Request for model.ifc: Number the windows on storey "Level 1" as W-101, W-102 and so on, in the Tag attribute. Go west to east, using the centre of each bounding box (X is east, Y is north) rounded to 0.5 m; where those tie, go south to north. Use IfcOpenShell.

First a look at what the model holds.

```python
import ifcopenshell
import ifcopenshell.util.element
import ifcopenshell.util.placement

model = ifcopenshell.open("model.ifc")
print(model.schema)
storey = next(s for s in model.by_type("IfcBuildingStorey") if s.Name == "Level 1")
windows = [e for e in ifcopenshell.util.element.get_decomposition(storey) if e.is_a("IfcWindow")]
for e in sorted(windows, key=lambda e: e.id()):
    origin = ifcopenshell.util.placement.get_local_placement(e.ObjectPlacement)[:3, 3]
    print(e.id(), e.Tag, e.Name, origin.round(2) + 0.0, sep=" | ")
```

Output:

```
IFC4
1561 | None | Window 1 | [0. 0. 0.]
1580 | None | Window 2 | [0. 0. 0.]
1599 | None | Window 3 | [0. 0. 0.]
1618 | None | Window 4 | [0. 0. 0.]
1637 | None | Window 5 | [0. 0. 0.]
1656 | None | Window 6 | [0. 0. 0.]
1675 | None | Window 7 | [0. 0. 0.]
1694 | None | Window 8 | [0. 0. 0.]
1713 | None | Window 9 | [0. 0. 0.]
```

```python
import ifcopenshell
import ifcopenshell.geom
import ifcopenshell.util.element
import ifcopenshell.util.shape

model = ifcopenshell.open("model.ifc")
settings = ifcopenshell.geom.settings()
settings.set("use-world-coords", True)


def centre(element):
    shape = ifcopenshell.geom.create_shape(settings, element)
    return ifcopenshell.util.shape.get_bbox_centroid(shape.geometry)


storey = next(s for s in model.by_type("IfcBuildingStorey") if s.Name == "Level 1")
windows = [e for e in ifcopenshell.util.element.get_decomposition(storey) if e.is_a("IfcWindow")]

# Insertion points can sit at a corner or the storey origin, so sort by the geometry (in metres).
centres = {e: centre(e) for e in windows}
windows.sort(key=lambda e: (round(centres[e][0] / 0.5), centres[e][1]))

for i, e in enumerate(windows, start=1):
    number = f"W-1{i:02d}"
    e.Tag = number
    print(e.id(), number)

model.write("model_updated.ifc")
```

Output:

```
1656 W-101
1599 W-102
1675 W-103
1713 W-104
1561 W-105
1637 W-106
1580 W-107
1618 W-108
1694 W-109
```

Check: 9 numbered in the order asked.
